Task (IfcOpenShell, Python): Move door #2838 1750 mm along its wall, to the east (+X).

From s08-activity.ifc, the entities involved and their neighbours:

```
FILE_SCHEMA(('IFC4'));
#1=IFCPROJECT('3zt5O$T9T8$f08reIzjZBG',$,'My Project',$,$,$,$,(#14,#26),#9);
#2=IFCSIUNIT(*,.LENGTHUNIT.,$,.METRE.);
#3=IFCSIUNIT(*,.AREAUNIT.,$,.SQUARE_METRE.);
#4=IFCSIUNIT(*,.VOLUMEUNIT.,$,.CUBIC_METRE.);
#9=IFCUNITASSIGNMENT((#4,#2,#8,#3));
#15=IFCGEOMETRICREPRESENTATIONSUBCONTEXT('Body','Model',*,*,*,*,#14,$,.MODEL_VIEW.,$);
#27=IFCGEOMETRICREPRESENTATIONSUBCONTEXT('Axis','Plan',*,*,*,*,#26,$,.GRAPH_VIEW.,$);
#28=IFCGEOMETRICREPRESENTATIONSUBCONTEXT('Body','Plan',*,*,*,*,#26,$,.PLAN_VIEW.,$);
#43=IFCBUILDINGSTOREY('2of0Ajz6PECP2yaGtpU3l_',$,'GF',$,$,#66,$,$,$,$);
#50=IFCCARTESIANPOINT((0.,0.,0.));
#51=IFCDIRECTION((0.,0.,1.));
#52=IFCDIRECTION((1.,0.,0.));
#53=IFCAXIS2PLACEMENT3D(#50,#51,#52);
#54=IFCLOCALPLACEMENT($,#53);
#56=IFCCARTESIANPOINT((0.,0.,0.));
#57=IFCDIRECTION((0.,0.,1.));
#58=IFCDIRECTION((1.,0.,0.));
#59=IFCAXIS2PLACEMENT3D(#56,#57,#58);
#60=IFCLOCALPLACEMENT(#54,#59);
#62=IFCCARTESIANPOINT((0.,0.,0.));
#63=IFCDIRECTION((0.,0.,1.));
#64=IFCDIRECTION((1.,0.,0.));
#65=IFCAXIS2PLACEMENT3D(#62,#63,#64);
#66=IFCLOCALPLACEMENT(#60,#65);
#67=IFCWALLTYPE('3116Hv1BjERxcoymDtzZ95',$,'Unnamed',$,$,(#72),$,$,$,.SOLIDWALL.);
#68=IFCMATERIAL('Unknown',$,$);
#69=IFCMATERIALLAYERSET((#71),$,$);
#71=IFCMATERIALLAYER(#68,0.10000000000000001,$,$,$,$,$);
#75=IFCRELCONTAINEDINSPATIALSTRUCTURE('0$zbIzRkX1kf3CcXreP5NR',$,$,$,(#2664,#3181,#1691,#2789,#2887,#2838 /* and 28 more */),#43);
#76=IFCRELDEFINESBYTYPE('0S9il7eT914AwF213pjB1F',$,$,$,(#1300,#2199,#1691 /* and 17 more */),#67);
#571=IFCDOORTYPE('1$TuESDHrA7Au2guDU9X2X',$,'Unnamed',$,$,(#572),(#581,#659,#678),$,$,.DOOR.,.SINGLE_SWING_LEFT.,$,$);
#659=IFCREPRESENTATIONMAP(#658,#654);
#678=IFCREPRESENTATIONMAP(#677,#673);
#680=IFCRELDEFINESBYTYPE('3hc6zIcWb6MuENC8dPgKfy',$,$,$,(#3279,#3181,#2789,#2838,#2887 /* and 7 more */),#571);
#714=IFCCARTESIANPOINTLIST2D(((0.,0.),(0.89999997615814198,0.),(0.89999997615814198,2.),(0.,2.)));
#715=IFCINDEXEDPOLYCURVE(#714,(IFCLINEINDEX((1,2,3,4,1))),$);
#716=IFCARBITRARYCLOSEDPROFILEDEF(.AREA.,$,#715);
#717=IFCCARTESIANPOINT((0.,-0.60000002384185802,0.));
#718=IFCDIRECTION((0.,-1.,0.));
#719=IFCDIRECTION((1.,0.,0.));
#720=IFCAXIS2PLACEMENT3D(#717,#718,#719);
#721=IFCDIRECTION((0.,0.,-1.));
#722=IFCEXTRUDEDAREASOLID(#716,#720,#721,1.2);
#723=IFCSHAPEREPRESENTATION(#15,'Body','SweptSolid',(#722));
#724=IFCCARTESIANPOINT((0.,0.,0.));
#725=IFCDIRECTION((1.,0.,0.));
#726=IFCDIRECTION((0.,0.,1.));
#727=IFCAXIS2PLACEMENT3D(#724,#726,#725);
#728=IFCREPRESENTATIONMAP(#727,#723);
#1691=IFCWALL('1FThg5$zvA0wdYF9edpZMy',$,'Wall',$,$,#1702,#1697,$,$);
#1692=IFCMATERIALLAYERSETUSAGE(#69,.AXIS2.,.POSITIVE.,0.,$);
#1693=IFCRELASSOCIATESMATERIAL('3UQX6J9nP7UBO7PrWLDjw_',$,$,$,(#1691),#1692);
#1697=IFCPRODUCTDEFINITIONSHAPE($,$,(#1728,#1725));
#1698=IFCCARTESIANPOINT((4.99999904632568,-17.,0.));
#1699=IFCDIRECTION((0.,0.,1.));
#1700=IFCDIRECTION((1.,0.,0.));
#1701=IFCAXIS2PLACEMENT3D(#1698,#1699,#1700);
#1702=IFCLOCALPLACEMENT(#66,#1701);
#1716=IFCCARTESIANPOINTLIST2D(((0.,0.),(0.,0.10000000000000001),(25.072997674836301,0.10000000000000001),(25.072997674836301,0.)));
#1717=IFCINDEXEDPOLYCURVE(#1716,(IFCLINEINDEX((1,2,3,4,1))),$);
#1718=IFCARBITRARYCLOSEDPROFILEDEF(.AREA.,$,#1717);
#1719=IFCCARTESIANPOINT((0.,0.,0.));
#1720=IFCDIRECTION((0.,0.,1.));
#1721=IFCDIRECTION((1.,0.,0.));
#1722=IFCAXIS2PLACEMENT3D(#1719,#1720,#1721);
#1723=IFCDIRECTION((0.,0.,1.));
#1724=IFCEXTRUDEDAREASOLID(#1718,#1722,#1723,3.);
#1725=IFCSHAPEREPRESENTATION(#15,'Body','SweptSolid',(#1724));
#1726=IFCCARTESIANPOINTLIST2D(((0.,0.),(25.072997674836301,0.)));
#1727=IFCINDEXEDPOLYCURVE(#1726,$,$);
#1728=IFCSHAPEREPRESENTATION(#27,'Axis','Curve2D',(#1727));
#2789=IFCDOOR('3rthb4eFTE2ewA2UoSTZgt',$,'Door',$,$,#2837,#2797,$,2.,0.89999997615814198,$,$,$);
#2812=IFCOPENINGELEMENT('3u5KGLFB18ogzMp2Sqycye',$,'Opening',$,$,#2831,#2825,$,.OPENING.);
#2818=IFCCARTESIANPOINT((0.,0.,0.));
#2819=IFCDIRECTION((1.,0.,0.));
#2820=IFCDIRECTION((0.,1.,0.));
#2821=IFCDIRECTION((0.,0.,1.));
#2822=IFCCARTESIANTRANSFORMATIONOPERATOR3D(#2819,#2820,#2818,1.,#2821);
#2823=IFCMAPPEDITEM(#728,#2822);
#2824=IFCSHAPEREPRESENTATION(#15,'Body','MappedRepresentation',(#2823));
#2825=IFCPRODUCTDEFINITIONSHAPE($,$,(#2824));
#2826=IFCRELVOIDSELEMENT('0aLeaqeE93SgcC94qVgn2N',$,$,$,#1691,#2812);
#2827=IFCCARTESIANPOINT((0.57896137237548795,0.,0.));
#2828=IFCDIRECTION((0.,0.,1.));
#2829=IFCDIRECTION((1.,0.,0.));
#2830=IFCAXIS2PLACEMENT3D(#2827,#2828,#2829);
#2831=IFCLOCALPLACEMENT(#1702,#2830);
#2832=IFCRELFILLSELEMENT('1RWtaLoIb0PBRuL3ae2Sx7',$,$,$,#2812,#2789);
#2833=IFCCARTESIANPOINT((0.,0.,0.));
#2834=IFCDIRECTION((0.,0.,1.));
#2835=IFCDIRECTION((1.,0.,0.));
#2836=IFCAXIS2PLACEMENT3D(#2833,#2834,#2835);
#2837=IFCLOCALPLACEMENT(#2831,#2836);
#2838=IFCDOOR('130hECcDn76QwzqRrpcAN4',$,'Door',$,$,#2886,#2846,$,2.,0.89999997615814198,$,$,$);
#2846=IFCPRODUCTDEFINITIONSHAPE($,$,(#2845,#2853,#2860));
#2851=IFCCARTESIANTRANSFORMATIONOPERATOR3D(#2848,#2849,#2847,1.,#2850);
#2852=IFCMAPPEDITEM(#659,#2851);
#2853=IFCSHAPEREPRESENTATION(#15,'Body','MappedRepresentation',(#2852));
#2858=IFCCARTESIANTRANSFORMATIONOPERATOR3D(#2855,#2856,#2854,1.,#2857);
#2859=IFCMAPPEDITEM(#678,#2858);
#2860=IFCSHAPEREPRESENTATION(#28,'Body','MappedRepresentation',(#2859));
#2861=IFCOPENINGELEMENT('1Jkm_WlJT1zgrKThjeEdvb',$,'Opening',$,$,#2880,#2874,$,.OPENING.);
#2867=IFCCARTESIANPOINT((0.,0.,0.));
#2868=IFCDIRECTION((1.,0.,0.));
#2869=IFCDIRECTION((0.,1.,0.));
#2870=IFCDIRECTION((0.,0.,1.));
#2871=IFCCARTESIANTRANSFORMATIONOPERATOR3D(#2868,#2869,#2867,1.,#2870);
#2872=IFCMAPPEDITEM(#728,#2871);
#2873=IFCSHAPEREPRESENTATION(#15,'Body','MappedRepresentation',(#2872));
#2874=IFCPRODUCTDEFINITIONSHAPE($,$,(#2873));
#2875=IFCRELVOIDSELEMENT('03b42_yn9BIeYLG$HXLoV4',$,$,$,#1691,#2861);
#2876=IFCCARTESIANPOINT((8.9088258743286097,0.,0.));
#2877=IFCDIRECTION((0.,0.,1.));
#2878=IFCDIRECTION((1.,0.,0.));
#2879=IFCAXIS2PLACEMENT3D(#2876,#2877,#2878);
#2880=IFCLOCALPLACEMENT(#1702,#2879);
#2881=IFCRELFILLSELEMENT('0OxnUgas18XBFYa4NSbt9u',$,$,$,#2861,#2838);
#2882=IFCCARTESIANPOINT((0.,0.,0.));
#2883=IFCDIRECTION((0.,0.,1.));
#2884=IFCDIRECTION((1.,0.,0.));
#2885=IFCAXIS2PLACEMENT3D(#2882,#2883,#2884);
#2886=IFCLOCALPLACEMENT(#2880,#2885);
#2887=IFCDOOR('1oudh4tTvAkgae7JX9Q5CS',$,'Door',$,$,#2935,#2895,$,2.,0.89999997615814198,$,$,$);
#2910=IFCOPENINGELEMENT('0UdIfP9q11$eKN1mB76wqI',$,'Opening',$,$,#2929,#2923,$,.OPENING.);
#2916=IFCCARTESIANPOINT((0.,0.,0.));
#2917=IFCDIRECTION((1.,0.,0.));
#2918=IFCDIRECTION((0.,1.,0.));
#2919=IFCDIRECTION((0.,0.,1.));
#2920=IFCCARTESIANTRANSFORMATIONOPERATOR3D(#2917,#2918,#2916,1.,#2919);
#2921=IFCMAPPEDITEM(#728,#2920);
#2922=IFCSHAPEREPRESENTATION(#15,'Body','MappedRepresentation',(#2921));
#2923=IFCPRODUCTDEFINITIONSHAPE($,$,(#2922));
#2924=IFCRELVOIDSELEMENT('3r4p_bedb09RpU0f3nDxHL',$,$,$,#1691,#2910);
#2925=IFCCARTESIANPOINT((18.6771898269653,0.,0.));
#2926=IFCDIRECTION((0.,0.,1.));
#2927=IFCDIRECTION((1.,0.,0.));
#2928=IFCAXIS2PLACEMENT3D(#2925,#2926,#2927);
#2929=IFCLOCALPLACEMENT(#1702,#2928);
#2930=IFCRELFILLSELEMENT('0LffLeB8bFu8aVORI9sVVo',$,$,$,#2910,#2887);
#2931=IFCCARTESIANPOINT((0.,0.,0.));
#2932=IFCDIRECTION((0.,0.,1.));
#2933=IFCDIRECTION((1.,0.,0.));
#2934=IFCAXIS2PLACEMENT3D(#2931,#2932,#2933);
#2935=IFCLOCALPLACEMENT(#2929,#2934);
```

```python
import ifcopenshell
import ifcopenshell.api.geometry
import ifcopenshell.util.placement
import ifcopenshell.util.unit

model = ifcopenshell.open("s08-activity.ifc")
unit_scale = ifcopenshell.util.unit.calculate_unit_scale(model)

door = model.by_guid("130hECcDn76QwzqRrpcAN4")
opening = door.FillsVoids[0].RelatingOpeningElement
wall = opening.VoidsElements[0].RelatingBuildingElement

wall_matrix = ifcopenshell.util.placement.get_local_placement(wall.ObjectPlacement)
shift = wall_matrix[:3, 0] * 1.75 / unit_scale
before = ifcopenshell.util.placement.get_local_placement(door.ObjectPlacement)[:3, 3].copy()

# The door is placed relative to its opening, so it follows when the opening moves.
matrix = ifcopenshell.util.placement.get_local_placement(opening.ObjectPlacement)
matrix[:3, 3] += shift
ifcopenshell.api.geometry.edit_object_placement(
    model, product=opening, matrix=matrix, is_si=False, should_transform_children=True
)

after = ifcopenshell.util.placement.get_local_placement(door.ObjectPlacement)[:3, 3]
print("door moved by", (after - before).round(3) + 0.0)

model.write("s08-activity-out.ifc")
```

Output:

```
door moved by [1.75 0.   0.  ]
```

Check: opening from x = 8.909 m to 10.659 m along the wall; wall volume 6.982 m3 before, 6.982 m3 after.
